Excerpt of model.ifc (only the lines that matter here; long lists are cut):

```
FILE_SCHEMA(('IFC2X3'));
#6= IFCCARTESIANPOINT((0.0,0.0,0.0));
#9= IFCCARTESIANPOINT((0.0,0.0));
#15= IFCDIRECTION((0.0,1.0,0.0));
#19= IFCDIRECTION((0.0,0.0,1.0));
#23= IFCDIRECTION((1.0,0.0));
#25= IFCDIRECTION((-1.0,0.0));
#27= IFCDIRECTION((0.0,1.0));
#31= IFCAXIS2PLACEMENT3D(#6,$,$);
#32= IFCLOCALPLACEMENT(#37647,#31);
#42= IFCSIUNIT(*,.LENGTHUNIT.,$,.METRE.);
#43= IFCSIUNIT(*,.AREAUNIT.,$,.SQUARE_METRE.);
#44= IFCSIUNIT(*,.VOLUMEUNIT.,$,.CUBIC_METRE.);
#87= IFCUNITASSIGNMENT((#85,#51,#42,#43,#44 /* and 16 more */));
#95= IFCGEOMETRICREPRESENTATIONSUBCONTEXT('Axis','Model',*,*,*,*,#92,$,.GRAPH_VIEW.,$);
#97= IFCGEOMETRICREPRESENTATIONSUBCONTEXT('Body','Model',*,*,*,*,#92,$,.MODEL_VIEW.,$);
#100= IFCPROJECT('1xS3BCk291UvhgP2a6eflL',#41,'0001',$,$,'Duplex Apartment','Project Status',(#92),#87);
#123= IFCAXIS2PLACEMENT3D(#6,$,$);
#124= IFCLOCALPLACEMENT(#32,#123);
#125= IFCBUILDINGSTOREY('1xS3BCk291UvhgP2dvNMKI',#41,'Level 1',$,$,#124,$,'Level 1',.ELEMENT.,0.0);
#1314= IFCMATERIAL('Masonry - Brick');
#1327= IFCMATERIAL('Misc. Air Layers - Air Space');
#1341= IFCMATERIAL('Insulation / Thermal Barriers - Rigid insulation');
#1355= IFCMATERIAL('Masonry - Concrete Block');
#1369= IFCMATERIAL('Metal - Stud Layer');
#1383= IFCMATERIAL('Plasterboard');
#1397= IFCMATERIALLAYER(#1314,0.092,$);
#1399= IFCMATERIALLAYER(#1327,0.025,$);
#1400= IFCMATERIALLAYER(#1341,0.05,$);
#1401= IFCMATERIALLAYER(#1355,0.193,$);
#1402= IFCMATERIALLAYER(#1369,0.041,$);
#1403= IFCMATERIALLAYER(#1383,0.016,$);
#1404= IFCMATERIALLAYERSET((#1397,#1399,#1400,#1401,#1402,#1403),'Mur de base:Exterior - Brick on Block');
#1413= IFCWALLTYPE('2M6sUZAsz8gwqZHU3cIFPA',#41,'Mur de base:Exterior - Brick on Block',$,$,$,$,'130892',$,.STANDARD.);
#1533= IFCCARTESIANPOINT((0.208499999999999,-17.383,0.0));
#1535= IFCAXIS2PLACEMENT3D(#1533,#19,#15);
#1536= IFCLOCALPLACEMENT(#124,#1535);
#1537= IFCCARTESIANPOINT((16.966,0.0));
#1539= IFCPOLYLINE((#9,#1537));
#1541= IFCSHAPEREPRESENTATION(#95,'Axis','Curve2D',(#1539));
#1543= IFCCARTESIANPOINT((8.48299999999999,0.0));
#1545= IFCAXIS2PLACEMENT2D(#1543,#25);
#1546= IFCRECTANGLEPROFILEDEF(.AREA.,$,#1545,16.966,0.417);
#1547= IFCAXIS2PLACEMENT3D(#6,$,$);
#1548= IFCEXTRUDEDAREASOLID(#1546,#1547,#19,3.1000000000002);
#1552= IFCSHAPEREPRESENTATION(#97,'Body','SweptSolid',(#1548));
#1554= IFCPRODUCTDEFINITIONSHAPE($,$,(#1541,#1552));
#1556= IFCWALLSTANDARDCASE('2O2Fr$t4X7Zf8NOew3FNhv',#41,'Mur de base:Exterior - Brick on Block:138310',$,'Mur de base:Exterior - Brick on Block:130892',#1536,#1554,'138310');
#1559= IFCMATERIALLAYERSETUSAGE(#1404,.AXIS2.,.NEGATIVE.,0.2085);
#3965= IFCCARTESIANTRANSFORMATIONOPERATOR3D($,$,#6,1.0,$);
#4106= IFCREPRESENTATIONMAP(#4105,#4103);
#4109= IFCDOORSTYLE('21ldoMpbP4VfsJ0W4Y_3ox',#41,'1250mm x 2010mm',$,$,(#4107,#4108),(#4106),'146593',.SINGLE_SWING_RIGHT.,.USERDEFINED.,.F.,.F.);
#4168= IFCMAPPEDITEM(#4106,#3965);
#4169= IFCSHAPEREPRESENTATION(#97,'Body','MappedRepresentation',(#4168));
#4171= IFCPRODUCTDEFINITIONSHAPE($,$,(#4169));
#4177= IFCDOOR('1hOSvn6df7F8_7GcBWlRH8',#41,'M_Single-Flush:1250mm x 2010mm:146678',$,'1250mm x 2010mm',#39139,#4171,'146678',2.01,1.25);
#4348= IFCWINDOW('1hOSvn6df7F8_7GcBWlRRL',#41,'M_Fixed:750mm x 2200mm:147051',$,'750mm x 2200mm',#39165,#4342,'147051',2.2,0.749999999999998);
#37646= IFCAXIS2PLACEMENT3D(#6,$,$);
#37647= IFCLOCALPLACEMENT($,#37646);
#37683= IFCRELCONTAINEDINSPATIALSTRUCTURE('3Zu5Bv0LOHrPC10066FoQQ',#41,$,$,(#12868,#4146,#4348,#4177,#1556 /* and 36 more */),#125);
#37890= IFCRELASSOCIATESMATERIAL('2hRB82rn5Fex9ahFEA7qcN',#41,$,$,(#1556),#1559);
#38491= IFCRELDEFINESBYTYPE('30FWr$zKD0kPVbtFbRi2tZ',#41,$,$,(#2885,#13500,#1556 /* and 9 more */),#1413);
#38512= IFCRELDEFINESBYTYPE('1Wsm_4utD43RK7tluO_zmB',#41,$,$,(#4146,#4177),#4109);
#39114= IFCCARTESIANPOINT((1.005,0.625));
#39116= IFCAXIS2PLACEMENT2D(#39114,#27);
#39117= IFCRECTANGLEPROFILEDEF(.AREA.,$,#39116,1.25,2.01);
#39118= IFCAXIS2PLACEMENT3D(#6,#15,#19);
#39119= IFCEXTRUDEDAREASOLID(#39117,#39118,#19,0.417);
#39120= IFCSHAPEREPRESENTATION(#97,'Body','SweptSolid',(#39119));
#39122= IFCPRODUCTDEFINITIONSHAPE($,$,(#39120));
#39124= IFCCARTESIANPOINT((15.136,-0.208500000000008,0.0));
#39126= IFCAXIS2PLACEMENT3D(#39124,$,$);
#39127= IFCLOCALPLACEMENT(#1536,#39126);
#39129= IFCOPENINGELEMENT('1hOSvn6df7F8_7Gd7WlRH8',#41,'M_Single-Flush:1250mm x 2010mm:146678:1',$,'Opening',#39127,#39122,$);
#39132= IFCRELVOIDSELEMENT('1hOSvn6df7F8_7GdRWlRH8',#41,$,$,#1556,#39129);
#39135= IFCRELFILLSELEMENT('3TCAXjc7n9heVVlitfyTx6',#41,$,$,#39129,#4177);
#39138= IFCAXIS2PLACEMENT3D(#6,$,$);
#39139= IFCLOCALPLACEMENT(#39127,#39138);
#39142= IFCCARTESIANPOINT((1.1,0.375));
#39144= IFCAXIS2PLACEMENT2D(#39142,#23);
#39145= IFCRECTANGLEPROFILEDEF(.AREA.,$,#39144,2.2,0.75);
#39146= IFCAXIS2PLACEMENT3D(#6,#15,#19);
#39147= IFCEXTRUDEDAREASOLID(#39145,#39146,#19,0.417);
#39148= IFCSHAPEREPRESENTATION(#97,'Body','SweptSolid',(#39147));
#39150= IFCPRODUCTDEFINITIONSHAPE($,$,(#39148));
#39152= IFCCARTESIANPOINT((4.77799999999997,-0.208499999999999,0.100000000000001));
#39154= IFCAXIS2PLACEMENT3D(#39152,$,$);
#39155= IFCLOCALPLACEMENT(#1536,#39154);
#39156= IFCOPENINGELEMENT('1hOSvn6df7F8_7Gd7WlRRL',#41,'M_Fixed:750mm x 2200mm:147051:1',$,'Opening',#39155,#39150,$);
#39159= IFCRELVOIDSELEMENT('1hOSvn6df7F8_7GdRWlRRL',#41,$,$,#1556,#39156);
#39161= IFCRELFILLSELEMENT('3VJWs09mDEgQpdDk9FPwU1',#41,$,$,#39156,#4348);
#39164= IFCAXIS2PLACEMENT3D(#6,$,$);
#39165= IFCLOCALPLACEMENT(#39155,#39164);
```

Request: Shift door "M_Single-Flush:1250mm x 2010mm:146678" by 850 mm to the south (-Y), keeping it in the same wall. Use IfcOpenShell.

```python
import ifcopenshell
import ifcopenshell.api.geometry
import ifcopenshell.util.placement

model = ifcopenshell.open("model.ifc")

door = model.by_guid("1hOSvn6df7F8_7GcBWlRH8")
opening = door.FillsVoids[0].RelatingOpeningElement
wall = opening.VoidsElements[0].RelatingBuildingElement

wall_matrix = ifcopenshell.util.placement.get_local_placement(wall.ObjectPlacement)
shift = wall_matrix[:3, 0] * -0.85
before = ifcopenshell.util.placement.get_local_placement(door.ObjectPlacement)[:3, 3].copy()

# The door is placed relative to its opening, so it follows when the opening moves.
matrix = ifcopenshell.util.placement.get_local_placement(opening.ObjectPlacement)
matrix[:3, 3] += shift
ifcopenshell.api.geometry.edit_object_placement(
    model, product=opening, matrix=matrix, is_si=False, should_transform_children=True
)

after = ifcopenshell.util.placement.get_local_placement(door.ObjectPlacement)[:3, 3]
print("door moved by", (after - before).round(3) + 0.0)

model.write("model-out.ifc")
```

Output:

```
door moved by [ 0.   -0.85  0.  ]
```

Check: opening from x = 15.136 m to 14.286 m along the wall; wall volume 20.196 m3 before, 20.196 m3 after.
